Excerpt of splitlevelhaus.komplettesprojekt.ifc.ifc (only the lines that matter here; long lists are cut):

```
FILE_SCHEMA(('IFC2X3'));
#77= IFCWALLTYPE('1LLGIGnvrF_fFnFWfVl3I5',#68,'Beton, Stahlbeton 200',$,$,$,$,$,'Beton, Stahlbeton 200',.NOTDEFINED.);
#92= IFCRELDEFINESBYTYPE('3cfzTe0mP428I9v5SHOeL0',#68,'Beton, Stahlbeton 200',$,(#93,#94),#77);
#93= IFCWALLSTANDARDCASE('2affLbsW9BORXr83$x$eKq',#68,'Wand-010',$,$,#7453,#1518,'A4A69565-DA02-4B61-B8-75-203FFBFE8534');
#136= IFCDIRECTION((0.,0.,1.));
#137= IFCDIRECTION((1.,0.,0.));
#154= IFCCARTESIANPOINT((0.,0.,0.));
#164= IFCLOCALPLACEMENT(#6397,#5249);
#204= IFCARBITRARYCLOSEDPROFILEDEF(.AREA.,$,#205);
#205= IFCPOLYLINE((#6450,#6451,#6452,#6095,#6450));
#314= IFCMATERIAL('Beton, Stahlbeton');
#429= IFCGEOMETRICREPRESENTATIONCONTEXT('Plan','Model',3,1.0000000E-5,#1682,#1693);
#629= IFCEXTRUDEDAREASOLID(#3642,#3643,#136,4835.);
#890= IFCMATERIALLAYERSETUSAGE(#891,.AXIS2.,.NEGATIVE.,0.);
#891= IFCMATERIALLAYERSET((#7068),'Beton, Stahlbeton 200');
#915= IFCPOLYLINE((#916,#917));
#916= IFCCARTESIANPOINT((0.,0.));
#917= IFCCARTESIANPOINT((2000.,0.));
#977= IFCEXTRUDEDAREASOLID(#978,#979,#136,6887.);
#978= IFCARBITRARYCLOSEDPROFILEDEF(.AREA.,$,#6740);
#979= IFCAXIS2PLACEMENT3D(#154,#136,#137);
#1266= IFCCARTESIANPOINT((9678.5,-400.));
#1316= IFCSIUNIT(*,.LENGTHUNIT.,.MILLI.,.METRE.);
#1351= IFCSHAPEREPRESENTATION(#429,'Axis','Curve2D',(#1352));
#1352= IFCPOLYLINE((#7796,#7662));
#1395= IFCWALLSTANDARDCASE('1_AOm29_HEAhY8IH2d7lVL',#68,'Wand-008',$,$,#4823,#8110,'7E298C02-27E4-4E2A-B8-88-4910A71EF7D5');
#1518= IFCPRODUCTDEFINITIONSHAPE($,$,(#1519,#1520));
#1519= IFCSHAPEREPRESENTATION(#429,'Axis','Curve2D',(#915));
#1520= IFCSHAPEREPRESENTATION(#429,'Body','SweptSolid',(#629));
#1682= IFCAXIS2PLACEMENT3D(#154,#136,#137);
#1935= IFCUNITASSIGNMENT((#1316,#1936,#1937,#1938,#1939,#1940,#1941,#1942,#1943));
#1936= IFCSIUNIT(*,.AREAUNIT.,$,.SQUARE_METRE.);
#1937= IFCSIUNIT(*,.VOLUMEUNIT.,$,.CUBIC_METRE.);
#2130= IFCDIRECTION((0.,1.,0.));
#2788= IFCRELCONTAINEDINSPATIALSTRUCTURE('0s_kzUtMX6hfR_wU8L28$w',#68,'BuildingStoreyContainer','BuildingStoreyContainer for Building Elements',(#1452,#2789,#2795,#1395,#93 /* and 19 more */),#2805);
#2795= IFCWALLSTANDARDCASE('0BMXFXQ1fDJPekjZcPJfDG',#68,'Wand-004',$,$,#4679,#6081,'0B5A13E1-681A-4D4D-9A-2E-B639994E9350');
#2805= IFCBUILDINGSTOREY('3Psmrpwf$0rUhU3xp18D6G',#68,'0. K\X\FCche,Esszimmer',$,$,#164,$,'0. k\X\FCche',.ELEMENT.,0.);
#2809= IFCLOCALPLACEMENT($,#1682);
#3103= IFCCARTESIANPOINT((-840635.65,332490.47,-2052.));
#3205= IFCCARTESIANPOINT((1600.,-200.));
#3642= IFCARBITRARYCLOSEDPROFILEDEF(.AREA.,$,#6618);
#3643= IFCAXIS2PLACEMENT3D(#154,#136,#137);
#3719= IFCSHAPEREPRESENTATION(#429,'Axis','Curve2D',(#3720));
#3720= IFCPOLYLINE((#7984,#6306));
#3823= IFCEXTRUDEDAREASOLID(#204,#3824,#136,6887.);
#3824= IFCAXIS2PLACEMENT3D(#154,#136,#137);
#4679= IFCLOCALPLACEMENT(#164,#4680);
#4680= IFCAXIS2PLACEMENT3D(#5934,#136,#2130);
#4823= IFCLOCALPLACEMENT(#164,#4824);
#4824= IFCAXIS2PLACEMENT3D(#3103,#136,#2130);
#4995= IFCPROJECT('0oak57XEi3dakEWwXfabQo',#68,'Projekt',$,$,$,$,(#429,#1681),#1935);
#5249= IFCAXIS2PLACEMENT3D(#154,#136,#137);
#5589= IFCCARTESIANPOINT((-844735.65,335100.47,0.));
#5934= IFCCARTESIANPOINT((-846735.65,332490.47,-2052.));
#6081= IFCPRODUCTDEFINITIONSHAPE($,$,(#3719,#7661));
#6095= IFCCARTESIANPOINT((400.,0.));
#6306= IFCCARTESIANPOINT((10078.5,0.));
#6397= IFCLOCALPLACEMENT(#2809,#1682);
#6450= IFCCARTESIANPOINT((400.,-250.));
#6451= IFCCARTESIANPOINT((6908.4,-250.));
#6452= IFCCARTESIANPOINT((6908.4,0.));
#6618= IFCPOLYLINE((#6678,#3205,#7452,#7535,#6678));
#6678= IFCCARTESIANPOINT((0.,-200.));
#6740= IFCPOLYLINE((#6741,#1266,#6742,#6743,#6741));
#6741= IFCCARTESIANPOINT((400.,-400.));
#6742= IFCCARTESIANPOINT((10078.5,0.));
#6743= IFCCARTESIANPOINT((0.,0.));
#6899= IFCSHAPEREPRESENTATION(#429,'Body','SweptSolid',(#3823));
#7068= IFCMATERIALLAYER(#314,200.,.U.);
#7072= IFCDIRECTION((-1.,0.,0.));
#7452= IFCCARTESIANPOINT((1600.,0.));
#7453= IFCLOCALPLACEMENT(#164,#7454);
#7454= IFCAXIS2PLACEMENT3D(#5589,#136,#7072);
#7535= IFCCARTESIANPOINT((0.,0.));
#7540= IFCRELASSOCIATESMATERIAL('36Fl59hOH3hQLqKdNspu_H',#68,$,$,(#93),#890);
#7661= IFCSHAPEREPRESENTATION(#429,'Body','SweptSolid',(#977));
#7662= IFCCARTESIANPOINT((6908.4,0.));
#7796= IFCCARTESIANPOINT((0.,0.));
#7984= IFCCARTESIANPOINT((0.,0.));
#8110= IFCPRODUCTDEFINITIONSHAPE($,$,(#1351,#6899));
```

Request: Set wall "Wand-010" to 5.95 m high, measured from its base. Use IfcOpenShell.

```python
import ifcopenshell
import ifcopenshell.geom
import ifcopenshell.util.shape
import ifcopenshell.util.unit

model = ifcopenshell.open("splitlevelhaus.komplettesprojekt.ifc.ifc")
unit_scale = ifcopenshell.util.unit.calculate_unit_scale(model)
settings = ifcopenshell.geom.settings()


def volume(element):
    """Net volume in cubic metres, openings subtracted."""
    shape = ifcopenshell.geom.create_shape(settings, element)
    return ifcopenshell.util.shape.get_volume(shape.geometry)


wall = model.by_guid("2affLbsW9BORXr83$x$eKq")
before = volume(wall)

body = next(r for r in wall.Representation.Representations if r.RepresentationIdentifier == "Body")
solid = body.Items[0]
old_height = solid.Depth
solid.Depth = 5.95 / unit_scale
after = volume(wall)

print(f"height {old_height:g} -> {solid.Depth:g}, volume {before:.3f} -> {after:.3f} m3")

model.write("splitlevelhaus.komplettesprojekt.ifc_edited.ifc")
```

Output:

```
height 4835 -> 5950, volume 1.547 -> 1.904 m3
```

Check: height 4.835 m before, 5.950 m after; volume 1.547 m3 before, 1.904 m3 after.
